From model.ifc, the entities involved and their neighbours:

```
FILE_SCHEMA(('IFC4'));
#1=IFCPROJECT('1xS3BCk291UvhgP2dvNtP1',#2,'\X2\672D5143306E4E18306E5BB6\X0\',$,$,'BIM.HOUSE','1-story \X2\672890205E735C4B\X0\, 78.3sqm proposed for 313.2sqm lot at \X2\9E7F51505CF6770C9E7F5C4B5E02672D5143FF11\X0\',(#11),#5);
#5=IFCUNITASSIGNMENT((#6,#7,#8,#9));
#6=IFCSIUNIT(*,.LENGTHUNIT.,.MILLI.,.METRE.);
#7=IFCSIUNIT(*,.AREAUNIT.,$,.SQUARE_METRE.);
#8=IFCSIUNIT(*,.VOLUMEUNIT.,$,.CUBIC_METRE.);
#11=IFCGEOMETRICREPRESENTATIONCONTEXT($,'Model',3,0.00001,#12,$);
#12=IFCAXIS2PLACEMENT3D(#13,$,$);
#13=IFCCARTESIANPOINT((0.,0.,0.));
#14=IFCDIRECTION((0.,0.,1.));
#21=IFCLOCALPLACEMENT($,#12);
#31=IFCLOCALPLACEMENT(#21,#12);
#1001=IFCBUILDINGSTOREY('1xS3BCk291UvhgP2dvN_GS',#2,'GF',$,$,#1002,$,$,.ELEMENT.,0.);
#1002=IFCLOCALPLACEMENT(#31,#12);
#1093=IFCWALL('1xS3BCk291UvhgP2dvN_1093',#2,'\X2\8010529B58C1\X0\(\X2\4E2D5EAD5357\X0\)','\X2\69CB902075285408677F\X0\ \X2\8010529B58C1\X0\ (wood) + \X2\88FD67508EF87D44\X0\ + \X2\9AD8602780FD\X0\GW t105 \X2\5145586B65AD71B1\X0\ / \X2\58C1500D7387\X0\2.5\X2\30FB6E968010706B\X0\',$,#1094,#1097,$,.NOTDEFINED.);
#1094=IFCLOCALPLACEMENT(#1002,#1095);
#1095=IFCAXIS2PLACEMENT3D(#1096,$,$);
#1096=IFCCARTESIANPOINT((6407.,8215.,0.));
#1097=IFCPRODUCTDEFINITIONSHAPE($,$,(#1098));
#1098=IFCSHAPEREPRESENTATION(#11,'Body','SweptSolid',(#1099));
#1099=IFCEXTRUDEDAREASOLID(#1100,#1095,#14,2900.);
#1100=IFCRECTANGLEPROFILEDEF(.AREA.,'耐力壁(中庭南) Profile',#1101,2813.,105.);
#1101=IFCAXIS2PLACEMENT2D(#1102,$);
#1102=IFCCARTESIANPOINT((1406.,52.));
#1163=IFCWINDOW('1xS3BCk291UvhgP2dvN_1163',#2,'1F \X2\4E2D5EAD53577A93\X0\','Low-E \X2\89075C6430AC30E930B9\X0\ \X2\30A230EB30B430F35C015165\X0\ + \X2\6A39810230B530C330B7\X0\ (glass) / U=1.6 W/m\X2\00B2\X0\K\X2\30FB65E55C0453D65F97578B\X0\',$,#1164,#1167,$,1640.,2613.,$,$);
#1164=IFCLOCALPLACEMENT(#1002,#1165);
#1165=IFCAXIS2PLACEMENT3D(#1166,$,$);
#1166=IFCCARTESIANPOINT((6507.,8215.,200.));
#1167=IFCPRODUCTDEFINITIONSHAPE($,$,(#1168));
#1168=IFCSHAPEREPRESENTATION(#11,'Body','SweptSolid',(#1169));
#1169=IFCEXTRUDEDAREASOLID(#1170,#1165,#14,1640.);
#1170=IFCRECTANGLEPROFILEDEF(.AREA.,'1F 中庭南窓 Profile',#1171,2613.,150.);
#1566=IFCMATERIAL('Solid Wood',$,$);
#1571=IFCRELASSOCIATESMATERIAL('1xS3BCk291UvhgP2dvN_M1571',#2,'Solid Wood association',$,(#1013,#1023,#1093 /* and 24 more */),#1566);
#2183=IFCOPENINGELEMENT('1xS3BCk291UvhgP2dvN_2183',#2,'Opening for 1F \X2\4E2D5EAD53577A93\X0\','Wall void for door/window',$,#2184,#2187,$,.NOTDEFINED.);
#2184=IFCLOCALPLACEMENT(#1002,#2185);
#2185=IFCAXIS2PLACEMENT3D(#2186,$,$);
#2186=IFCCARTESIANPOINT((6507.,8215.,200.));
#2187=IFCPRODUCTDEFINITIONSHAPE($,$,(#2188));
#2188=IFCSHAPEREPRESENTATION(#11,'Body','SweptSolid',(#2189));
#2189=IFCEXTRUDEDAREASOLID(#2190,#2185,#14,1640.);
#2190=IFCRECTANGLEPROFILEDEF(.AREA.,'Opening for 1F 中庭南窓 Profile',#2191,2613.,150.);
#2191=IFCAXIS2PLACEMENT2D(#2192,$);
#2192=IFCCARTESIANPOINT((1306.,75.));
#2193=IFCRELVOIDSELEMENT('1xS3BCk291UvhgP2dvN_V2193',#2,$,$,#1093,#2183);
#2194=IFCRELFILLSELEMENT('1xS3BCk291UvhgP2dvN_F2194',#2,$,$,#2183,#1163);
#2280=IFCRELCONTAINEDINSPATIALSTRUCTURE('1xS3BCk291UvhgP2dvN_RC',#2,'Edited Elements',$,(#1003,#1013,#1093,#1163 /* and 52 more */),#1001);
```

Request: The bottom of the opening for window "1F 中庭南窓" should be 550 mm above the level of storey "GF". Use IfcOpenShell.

```python
import numpy as np
import ifcopenshell
import ifcopenshell.api.geometry
import ifcopenshell.geom
import ifcopenshell.util.element
import ifcopenshell.util.placement
import ifcopenshell.util.shape
import ifcopenshell.util.unit

model = ifcopenshell.open("model.ifc")
unit_scale = ifcopenshell.util.unit.calculate_unit_scale(model)

window = model.by_id(1163)
opening = window.FillsVoids[0].RelatingOpeningElement
storey = ifcopenshell.util.element.get_container(window, ifc_class="IfcBuildingStorey")
level = ifcopenshell.util.placement.get_local_placement(storey.ObjectPlacement)[2, 3]

# The opening's origin need not be at the sill, so measure its lowest point.
shape = ifcopenshell.geom.create_shape(ifcopenshell.geom.settings(), opening)
bottom = ifcopenshell.util.shape.get_shape_bottom_elevation(shape, shape.geometry) / unit_scale
dz = level + 550.0 - bottom

shift = np.array([0.0, 0.0, dz])
# The window is not placed relative to its opening, so move both.
for product in (opening, window):
    matrix = ifcopenshell.util.placement.get_local_placement(product.ObjectPlacement)
    matrix[:3, 3] += shift
    ifcopenshell.api.geometry.edit_object_placement(model, product=product, matrix=matrix, is_si=False)

print(f"moved by {dz * unit_scale:+.3f} m")

model.write("model-out.ifc")
```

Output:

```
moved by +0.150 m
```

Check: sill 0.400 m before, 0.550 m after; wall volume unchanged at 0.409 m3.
